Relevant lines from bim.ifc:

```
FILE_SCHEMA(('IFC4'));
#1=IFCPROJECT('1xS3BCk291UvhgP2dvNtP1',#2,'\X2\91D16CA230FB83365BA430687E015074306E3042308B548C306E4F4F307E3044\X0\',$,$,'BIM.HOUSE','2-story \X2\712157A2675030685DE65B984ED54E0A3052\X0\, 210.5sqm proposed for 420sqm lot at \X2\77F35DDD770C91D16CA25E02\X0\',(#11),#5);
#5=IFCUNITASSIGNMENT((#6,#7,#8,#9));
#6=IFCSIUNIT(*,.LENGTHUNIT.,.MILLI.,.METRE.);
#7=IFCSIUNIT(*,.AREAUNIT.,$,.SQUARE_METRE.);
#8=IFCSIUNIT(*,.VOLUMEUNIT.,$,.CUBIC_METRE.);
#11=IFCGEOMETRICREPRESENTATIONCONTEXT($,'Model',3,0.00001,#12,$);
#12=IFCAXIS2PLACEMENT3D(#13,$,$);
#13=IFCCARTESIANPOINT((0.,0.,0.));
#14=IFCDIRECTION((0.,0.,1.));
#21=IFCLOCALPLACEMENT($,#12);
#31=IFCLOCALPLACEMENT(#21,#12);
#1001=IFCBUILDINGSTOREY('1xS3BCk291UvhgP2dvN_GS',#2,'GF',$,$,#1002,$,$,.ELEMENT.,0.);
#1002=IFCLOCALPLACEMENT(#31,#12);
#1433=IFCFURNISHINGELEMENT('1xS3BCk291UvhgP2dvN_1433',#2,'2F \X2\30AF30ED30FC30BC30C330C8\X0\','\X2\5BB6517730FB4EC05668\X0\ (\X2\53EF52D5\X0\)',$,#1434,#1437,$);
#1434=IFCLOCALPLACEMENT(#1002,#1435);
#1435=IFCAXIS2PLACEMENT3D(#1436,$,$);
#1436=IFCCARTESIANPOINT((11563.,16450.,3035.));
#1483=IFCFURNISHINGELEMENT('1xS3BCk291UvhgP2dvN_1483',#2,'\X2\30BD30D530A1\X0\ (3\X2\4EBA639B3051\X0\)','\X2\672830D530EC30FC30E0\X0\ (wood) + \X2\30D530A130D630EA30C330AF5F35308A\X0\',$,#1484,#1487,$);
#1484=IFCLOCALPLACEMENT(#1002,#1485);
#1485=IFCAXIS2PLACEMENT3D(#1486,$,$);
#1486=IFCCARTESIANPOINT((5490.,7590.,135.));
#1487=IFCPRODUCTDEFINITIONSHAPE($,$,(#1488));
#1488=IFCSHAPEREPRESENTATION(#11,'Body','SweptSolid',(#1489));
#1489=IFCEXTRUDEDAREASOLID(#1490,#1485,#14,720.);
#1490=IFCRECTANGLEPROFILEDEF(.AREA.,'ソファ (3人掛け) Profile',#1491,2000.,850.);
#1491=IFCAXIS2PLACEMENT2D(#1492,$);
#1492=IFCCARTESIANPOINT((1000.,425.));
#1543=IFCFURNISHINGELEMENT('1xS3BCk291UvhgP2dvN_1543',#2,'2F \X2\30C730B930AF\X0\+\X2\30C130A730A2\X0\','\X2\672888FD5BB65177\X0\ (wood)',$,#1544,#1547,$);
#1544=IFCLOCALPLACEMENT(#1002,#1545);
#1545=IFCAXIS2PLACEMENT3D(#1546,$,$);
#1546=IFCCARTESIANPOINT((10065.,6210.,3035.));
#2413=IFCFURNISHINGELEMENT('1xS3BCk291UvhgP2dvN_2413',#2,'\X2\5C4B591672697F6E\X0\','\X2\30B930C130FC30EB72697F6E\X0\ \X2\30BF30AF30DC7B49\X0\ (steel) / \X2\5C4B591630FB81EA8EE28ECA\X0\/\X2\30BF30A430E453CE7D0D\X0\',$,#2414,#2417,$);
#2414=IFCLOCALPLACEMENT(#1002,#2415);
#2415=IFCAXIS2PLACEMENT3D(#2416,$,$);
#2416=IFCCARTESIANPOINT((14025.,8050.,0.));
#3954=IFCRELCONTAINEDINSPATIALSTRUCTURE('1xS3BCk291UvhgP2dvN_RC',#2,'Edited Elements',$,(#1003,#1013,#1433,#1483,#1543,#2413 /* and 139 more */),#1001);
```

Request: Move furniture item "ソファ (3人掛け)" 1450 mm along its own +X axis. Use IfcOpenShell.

```python
import ifcopenshell
import ifcopenshell.api.geometry
import ifcopenshell.util.placement

model = ifcopenshell.open("bim.ifc")

item = model.by_guid("1xS3BCk291UvhgP2dvN_1483")
matrix = ifcopenshell.util.placement.get_local_placement(item.ObjectPlacement)
matrix[:3, 3] += matrix[:3, 0] * 1450.0
ifcopenshell.api.geometry.edit_object_placement(model, product=item, matrix=matrix, is_si=False)

print(ifcopenshell.util.placement.get_local_placement(item.ObjectPlacement).round(3) + 0.0)

model.write("bim_v2.ifc")
```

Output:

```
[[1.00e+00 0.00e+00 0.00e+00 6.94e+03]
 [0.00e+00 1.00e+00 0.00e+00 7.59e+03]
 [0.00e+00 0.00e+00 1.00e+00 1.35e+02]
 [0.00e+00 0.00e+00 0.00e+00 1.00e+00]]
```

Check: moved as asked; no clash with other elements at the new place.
